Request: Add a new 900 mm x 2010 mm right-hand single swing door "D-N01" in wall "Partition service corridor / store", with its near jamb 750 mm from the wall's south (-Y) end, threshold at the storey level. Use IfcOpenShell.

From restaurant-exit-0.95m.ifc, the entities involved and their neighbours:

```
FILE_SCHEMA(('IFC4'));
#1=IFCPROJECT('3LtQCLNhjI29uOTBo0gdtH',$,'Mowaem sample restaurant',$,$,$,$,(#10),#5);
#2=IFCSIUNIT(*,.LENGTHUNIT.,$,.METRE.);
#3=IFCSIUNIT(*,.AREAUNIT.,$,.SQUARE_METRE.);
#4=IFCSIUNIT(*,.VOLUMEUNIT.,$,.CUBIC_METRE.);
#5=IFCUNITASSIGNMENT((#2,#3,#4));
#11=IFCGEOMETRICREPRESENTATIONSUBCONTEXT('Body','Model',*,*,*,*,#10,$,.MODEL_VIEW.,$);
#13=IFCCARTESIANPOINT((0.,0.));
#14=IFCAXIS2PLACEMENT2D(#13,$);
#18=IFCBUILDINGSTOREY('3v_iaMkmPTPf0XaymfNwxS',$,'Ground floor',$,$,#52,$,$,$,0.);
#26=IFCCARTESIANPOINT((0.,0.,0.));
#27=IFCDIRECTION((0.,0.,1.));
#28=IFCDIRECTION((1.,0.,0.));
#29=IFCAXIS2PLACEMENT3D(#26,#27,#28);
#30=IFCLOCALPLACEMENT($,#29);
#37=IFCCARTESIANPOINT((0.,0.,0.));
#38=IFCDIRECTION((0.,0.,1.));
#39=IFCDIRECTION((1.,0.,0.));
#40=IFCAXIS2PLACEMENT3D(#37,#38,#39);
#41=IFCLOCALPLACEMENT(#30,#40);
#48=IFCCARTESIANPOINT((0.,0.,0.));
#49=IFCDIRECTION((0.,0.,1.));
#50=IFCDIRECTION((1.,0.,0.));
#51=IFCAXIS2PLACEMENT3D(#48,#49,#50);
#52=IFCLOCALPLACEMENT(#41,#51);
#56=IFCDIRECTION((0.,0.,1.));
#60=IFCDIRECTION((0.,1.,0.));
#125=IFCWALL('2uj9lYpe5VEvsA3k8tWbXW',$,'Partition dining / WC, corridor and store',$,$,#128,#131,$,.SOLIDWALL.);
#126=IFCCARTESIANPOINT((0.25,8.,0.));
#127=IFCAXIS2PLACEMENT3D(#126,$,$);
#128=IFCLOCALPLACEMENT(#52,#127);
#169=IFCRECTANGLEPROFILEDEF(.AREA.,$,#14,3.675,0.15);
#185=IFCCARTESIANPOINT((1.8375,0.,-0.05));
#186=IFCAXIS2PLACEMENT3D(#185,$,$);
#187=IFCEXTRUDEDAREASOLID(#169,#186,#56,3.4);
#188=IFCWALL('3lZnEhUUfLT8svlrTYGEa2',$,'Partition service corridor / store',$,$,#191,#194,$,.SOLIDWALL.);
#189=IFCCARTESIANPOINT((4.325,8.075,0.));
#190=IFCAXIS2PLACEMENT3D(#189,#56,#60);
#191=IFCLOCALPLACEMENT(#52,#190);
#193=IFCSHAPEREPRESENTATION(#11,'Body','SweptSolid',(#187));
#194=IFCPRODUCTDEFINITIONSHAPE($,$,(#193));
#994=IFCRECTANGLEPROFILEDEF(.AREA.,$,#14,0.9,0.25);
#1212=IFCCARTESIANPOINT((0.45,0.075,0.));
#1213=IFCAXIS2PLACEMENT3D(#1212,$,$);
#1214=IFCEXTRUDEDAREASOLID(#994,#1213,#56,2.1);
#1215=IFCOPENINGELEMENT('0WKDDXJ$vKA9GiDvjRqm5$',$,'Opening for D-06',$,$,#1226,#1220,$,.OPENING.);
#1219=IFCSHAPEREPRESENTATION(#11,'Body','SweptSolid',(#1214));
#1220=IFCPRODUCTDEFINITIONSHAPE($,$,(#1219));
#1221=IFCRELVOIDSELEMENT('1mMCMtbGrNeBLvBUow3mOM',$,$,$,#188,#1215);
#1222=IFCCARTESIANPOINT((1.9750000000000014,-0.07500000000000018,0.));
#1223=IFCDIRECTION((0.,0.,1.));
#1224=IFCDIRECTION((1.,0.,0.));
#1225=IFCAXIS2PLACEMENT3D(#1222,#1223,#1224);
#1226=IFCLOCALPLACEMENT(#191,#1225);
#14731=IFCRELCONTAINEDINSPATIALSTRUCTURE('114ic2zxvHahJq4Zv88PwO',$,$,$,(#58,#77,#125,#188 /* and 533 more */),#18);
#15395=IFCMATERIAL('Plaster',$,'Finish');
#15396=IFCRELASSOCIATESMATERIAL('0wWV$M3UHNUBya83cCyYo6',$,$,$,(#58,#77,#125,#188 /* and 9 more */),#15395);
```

```python
import numpy as np
import ifcopenshell
import ifcopenshell.api.feature
import ifcopenshell.api.geometry
import ifcopenshell.api.root
import ifcopenshell.api.spatial
import ifcopenshell.geom
import ifcopenshell.util.element
import ifcopenshell.util.placement
import ifcopenshell.util.representation
import ifcopenshell.util.shape
import ifcopenshell.util.unit

model = ifcopenshell.open("restaurant-exit-0.95m.ifc")
unit_scale = ifcopenshell.util.unit.calculate_unit_scale(model)
settings = ifcopenshell.geom.settings()


def volume(element):
    """Net volume in cubic metres, openings subtracted."""
    shape = ifcopenshell.geom.create_shape(settings, element)
    return ifcopenshell.util.shape.get_volume(shape.geometry)


wall = model.by_id(188)
storey = ifcopenshell.util.element.get_container(wall, ifc_class="IfcBuildingStorey")
context = ifcopenshell.util.representation.get_context(model, "Model", "Body", "MODEL_VIEW")
before = volume(wall)

width, height, from_end, sill = 0.9, 2.01, 0.75, 0.0  # metres

# The wall runs along its own X axis, and the end named is its -X end.
wall_shape = ifcopenshell.geom.create_shape(settings, wall)
x, y, z = ifcopenshell.util.shape.get_vertices(wall_shape.geometry).T
start = x.min() + from_end
face, thickness = float(y.min()), float(y.max() - y.min())
wall_matrix = ifcopenshell.util.placement.get_local_placement(wall.ObjectPlacement)
level = ifcopenshell.util.placement.get_local_placement(storey.ObjectPlacement)[2, 3]


def in_wall(x, y):
    """Placement at x, y metres in the wall's axes, at sill height."""
    matrix = wall_matrix.copy()
    matrix[:, 3] = wall_matrix @ np.array([x / unit_scale, y / unit_scale, 0.0, 1.0])
    matrix[2, 3] = level + sill / unit_scale
    return matrix


# Opening: a box that overshoots both wall faces by 50 mm.
opening = ifcopenshell.api.root.create_entity(model, ifc_class="IfcOpeningElement", predefined_type="OPENING")
box = ifcopenshell.api.geometry.add_wall_representation(
    model, context=context, length=width, height=height, thickness=thickness + 0.1
)
ifcopenshell.api.geometry.assign_representation(model, product=opening, representation=box)
ifcopenshell.api.geometry.edit_object_placement(model, product=opening, matrix=in_wall(start, face - 0.05), is_si=False)
ifcopenshell.api.feature.add_feature(model, feature=opening, element=wall)

door = ifcopenshell.api.root.create_entity(model, ifc_class="IfcDoor", name="D-N01", predefined_type="DOOR")
door.OverallWidth, door.OverallHeight = width / unit_scale, height / unit_scale
door.OperationType = "SINGLE_SWING_RIGHT"
body = ifcopenshell.api.geometry.add_door_representation(
    model,
    context=context,
    overall_width=door.OverallWidth,
    overall_height=door.OverallHeight,
    operation_type="SINGLE_SWING_RIGHT",
    lining_properties={"LiningDepth": thickness / unit_scale, "ThresholdDepth": thickness / unit_scale},
)
ifcopenshell.api.geometry.assign_representation(model, product=door, representation=body)
ifcopenshell.api.spatial.assign_container(model, products=[door], relating_structure=storey)
ifcopenshell.api.feature.add_filling(model, opening=opening, element=door)

# The lining spans the wall, so the door starts at the wall face.
ifcopenshell.api.geometry.edit_object_placement(model, product=door, matrix=in_wall(start, face), is_si=False)

after = volume(wall)

print(f"wall volume {before:.3f} -> {after:.3f} m3")

model.write("restaurant-exit-0.95m_rev.ifc")
```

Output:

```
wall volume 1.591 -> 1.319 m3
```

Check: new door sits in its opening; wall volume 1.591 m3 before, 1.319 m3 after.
